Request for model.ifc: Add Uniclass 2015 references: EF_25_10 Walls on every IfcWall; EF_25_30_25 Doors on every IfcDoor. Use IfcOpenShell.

First a look at what the model holds.

```python
import ifcopenshell

model = ifcopenshell.open("model.ifc")
print(model.schema)
print("classifications:", [c.Name for c in model.by_type("IfcClassification")])
for ifc_class in ("IfcDoor", "IfcRoof", "IfcStair", "IfcWall", "IfcWindow"):
    print(ifc_class, len(model.by_type(ifc_class)))
```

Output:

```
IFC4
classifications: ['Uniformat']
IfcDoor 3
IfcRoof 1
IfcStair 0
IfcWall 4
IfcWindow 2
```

```python
import ifcopenshell
import ifcopenshell.api.classification

model = ifcopenshell.open("model.ifc")

system = ifcopenshell.api.classification.add_classification(model, classification="Uniclass 2015")

codes = {
    "IfcWall": ("EF_25_10", "Walls"),
    "IfcDoor": ("EF_25_30_25", "Doors"),
}
for ifc_class, (code, name) in codes.items():
    products = model.by_type(ifc_class)
    ifcopenshell.api.classification.add_reference(
        model, products=products, classification=system, identification=code, name=name
    )
    print(code, len(products))

model.write("model_edited.ifc")
```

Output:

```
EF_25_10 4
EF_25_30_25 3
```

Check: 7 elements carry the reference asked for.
